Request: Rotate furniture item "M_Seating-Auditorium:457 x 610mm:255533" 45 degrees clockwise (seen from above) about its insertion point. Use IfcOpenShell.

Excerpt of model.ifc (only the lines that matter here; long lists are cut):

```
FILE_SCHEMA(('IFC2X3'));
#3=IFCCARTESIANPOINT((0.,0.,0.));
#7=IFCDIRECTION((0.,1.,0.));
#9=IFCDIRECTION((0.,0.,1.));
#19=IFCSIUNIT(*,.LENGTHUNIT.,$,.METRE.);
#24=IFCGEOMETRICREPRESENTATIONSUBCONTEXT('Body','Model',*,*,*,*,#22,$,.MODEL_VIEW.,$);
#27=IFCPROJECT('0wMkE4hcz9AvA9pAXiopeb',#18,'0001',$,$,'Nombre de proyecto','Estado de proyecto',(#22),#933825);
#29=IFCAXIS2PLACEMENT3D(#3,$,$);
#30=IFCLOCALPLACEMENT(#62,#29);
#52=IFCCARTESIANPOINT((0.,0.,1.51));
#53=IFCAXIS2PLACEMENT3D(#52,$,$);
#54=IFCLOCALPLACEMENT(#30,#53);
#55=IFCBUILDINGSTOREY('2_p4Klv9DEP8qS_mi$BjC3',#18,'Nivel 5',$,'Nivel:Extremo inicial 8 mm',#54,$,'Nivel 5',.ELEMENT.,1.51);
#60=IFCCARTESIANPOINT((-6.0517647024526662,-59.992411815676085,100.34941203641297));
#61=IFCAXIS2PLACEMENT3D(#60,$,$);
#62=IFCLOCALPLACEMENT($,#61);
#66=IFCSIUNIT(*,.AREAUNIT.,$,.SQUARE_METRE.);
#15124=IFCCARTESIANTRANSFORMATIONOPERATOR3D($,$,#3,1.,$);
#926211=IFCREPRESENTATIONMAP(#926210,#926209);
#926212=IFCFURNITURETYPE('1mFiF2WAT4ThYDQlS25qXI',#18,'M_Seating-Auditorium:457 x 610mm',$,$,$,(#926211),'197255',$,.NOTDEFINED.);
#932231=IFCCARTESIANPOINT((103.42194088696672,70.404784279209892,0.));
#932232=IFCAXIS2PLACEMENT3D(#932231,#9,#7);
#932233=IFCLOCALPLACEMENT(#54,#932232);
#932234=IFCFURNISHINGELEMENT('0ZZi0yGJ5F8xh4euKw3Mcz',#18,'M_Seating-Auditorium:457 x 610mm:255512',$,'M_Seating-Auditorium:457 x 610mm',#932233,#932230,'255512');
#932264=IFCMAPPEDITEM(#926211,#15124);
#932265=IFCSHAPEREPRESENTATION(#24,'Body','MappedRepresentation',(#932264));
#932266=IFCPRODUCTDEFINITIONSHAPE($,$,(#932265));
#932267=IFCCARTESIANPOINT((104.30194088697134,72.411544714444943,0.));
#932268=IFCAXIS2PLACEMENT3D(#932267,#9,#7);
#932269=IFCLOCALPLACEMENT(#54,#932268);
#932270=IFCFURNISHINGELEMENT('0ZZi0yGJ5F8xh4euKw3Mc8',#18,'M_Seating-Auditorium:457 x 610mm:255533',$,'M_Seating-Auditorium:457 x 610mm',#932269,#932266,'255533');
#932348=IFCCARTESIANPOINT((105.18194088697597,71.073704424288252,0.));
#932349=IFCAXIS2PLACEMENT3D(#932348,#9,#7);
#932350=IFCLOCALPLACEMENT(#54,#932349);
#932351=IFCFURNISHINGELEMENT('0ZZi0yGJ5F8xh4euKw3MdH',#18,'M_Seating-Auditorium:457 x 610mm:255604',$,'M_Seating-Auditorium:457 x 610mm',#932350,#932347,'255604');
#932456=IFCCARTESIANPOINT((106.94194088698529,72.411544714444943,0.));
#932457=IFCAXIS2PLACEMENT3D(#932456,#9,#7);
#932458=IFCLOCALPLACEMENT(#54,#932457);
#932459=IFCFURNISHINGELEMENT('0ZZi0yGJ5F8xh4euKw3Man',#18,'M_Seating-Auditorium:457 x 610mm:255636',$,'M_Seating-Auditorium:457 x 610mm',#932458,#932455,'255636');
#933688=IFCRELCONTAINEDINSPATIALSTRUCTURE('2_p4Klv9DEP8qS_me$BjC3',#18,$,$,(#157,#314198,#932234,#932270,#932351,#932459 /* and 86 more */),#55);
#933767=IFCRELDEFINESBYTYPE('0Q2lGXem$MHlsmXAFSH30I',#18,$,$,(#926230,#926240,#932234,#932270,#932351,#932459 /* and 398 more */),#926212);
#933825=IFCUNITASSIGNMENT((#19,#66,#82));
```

```python
import ifcopenshell
import ifcopenshell.api.geometry
import ifcopenshell.util.placement

model = ifcopenshell.open("model.ifc")

item = model.by_id(932270)
matrix = ifcopenshell.util.placement.get_local_placement(item.ObjectPlacement)
matrix = matrix @ ifcopenshell.util.placement.rotation(-45, "Z")
ifcopenshell.api.geometry.edit_object_placement(model, product=item, matrix=matrix, is_si=False)

print(ifcopenshell.util.placement.get_local_placement(item.ObjectPlacement).round(3) + 0.0)

model.write("model_updated.ifc")
```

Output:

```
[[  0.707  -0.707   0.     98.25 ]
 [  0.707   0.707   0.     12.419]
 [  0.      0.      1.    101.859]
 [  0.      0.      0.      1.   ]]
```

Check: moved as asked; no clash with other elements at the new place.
